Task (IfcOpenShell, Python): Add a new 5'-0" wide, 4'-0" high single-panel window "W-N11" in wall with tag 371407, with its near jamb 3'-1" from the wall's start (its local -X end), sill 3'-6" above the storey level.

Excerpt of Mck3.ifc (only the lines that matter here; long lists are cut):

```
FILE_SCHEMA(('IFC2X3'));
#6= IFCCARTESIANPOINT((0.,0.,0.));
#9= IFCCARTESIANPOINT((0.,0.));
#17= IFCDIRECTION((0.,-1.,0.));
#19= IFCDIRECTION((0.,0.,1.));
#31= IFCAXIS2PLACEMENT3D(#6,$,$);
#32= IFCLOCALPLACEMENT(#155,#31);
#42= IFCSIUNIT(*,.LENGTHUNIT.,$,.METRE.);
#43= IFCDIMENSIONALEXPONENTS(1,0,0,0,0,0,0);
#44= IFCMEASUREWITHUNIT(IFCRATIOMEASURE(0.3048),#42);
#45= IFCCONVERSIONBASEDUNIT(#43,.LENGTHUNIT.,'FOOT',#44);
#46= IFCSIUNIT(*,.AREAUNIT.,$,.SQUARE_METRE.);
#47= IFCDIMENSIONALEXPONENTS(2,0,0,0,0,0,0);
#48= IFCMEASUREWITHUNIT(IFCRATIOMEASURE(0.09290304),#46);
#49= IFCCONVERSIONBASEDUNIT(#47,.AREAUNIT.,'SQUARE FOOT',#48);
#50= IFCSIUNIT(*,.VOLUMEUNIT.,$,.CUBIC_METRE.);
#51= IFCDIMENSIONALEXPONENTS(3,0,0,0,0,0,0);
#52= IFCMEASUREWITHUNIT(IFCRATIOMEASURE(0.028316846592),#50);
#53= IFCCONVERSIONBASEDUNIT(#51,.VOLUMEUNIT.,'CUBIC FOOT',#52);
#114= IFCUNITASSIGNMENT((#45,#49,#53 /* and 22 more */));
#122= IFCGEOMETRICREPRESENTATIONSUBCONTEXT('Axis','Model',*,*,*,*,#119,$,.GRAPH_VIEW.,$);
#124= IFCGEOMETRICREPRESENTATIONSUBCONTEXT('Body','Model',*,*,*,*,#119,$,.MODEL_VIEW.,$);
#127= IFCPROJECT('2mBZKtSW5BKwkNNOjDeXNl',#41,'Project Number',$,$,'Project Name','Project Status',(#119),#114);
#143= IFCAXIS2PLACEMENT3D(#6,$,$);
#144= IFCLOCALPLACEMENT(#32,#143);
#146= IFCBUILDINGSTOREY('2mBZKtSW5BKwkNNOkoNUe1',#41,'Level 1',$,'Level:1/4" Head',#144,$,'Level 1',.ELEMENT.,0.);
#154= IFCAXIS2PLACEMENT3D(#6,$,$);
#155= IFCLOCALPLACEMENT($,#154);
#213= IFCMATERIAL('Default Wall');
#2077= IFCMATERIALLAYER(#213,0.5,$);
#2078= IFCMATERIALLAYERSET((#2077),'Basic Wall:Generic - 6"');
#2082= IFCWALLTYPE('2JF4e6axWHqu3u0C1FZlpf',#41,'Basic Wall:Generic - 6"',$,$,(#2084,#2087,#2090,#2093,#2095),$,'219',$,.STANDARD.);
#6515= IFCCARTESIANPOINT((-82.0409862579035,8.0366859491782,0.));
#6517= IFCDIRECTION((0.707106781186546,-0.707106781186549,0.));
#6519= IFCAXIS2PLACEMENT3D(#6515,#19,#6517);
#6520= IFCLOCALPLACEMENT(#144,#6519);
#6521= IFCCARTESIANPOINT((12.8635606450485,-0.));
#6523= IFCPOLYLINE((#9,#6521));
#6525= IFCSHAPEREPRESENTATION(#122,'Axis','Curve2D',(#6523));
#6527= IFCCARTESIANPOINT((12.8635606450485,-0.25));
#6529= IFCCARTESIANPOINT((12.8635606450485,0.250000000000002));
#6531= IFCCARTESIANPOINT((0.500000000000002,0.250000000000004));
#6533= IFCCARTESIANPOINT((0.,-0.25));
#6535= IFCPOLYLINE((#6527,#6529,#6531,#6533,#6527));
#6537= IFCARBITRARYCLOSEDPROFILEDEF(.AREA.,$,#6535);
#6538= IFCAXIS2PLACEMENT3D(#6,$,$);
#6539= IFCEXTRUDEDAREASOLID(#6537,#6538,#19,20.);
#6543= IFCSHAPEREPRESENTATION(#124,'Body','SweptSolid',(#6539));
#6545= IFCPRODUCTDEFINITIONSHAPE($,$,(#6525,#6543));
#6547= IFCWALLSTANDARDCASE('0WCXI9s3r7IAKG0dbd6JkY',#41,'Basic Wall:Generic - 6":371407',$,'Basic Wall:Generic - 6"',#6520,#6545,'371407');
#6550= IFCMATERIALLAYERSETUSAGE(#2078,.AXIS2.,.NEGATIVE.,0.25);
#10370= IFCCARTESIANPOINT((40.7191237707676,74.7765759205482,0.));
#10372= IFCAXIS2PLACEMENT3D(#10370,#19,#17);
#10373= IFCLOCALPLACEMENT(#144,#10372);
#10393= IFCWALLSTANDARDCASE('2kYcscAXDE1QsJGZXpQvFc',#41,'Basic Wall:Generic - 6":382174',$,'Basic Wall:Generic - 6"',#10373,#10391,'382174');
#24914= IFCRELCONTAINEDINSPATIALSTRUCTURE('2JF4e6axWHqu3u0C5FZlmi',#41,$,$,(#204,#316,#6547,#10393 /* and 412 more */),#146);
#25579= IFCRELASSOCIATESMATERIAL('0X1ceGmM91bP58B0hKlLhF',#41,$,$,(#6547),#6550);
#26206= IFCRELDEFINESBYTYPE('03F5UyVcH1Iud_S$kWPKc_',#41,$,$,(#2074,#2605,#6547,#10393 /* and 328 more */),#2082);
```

```python
import numpy as np
import ifcopenshell
import ifcopenshell.api.feature
import ifcopenshell.api.geometry
import ifcopenshell.api.root
import ifcopenshell.api.spatial
import ifcopenshell.api.type
import ifcopenshell.geom
import ifcopenshell.util.element
import ifcopenshell.util.placement
import ifcopenshell.util.representation
import ifcopenshell.util.shape
import ifcopenshell.util.unit

model = ifcopenshell.open("Mck3.ifc")
unit_scale = ifcopenshell.util.unit.calculate_unit_scale(model)
settings = ifcopenshell.geom.settings()


def volume(element):
    """Net volume in cubic metres, openings subtracted."""
    shape = ifcopenshell.geom.create_shape(settings, element)
    return ifcopenshell.util.shape.get_volume(shape.geometry)


wall = model.by_guid("0WCXI9s3r7IAKG0dbd6JkY")
storey = ifcopenshell.util.element.get_container(wall, ifc_class="IfcBuildingStorey")
context = ifcopenshell.util.representation.get_context(model, "Model", "Body", "MODEL_VIEW")
before = volume(wall)

width, height, from_end, sill = 1.524, 1.2192, 0.9398, 1.0668  # metres

# The wall runs along its own X axis, and the end named is its -X end.
wall_shape = ifcopenshell.geom.create_shape(settings, wall)
x, y, z = ifcopenshell.util.shape.get_vertices(wall_shape.geometry).T
start = x.min() + from_end
face, thickness = float(y.min()), float(y.max() - y.min())
wall_matrix = ifcopenshell.util.placement.get_local_placement(wall.ObjectPlacement)
level = ifcopenshell.util.placement.get_local_placement(storey.ObjectPlacement)[2, 3]


def in_wall(x, y):
    """Placement at x, y metres in the wall's axes, at sill height."""
    matrix = wall_matrix.copy()
    matrix[:, 3] = wall_matrix @ np.array([x / unit_scale, y / unit_scale, 0.0, 1.0])
    matrix[2, 3] = level + sill / unit_scale
    return matrix


# Opening: a box that overshoots both wall faces by 50 mm.
opening = ifcopenshell.api.root.create_entity(model, ifc_class="IfcOpeningElement")
box = ifcopenshell.api.geometry.add_wall_representation(
    model, context=context, length=width, height=height, thickness=thickness + 0.1
)
ifcopenshell.api.geometry.assign_representation(model, product=opening, representation=box)
ifcopenshell.api.geometry.edit_object_placement(model, product=opening, matrix=in_wall(start, face - 0.05), is_si=False)
ifcopenshell.api.feature.add_feature(model, feature=opening, element=wall)

window = ifcopenshell.api.root.create_entity(model, ifc_class="IfcWindow", name="W-N11")
window.OverallWidth, window.OverallHeight = width / unit_scale, height / unit_scale
body = ifcopenshell.api.geometry.add_window_representation(
    model,
    context=context,
    overall_width=window.OverallWidth,
    overall_height=window.OverallHeight,
    partition_type="SINGLE_PANEL",
)
ifcopenshell.api.geometry.assign_representation(model, product=window, representation=body)
ifcopenshell.api.spatial.assign_container(model, products=[window], relating_structure=storey)
fills = ifcopenshell.api.feature.add_filling(model, opening=opening, element=window)
fills.OwnerHistory = window.OwnerHistory  # required in IFC2X3

# IFC2X3 keeps the operation on the window style.
style = ifcopenshell.api.root.create_entity(model, ifc_class="IfcWindowStyle", name="W-N11")
style.OperationType, style.ConstructionType = "SINGLE_PANEL", "NOTDEFINED"
style.ParameterTakesPrecedence = style.Sizeable = False
ifcopenshell.api.type.assign_type(model, related_objects=[window], relating_type=style)

# Centre the window in the wall's thickness.
ifcopenshell.api.geometry.edit_object_placement(model, product=window, matrix=in_wall(start, face), is_si=False)
window_shape = ifcopenshell.geom.create_shape(settings, window)
depth = ifcopenshell.util.shape.get_vertices(window_shape.geometry)[:, 1]
offset = face + thickness / 2 - (depth.min() + depth.max()) / 2
ifcopenshell.api.geometry.edit_object_placement(model, product=window, matrix=in_wall(start, offset), is_si=False)

after = volume(wall)

print(f"wall volume {before:.3f} -> {after:.3f} m3")

model.write("Mck3_updated.ifc")
```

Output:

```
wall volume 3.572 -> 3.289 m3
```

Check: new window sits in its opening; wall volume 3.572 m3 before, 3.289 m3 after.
